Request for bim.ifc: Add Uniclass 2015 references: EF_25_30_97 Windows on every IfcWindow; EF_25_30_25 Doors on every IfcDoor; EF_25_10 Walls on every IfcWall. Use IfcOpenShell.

First a look at what the model holds.

```python
import ifcopenshell

model = ifcopenshell.open("bim.ifc")
print(model.schema)
print("classifications:", [c.Name for c in model.by_type("IfcClassification")])
for ifc_class in ("IfcDoor", "IfcRoof", "IfcStair", "IfcWall", "IfcWindow"):
    print(ifc_class, len(model.by_type(ifc_class)))
```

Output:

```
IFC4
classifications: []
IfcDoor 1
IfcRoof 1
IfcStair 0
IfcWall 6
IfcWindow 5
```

```python
import ifcopenshell
import ifcopenshell.api.classification

model = ifcopenshell.open("bim.ifc")

system = ifcopenshell.api.classification.add_classification(model, classification="Uniclass 2015")

codes = {
    "IfcWindow": ("EF_25_30_97", "Windows"),
    "IfcDoor": ("EF_25_30_25", "Doors"),
    "IfcWall": ("EF_25_10", "Walls"),
}
for ifc_class, (code, name) in codes.items():
    products = model.by_type(ifc_class)
    ifcopenshell.api.classification.add_reference(
        model, products=products, classification=system, identification=code, name=name
    )
    print(code, len(products))

model.write("bim_edited.ifc")
```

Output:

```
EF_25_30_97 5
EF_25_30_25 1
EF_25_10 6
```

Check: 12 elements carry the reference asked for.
